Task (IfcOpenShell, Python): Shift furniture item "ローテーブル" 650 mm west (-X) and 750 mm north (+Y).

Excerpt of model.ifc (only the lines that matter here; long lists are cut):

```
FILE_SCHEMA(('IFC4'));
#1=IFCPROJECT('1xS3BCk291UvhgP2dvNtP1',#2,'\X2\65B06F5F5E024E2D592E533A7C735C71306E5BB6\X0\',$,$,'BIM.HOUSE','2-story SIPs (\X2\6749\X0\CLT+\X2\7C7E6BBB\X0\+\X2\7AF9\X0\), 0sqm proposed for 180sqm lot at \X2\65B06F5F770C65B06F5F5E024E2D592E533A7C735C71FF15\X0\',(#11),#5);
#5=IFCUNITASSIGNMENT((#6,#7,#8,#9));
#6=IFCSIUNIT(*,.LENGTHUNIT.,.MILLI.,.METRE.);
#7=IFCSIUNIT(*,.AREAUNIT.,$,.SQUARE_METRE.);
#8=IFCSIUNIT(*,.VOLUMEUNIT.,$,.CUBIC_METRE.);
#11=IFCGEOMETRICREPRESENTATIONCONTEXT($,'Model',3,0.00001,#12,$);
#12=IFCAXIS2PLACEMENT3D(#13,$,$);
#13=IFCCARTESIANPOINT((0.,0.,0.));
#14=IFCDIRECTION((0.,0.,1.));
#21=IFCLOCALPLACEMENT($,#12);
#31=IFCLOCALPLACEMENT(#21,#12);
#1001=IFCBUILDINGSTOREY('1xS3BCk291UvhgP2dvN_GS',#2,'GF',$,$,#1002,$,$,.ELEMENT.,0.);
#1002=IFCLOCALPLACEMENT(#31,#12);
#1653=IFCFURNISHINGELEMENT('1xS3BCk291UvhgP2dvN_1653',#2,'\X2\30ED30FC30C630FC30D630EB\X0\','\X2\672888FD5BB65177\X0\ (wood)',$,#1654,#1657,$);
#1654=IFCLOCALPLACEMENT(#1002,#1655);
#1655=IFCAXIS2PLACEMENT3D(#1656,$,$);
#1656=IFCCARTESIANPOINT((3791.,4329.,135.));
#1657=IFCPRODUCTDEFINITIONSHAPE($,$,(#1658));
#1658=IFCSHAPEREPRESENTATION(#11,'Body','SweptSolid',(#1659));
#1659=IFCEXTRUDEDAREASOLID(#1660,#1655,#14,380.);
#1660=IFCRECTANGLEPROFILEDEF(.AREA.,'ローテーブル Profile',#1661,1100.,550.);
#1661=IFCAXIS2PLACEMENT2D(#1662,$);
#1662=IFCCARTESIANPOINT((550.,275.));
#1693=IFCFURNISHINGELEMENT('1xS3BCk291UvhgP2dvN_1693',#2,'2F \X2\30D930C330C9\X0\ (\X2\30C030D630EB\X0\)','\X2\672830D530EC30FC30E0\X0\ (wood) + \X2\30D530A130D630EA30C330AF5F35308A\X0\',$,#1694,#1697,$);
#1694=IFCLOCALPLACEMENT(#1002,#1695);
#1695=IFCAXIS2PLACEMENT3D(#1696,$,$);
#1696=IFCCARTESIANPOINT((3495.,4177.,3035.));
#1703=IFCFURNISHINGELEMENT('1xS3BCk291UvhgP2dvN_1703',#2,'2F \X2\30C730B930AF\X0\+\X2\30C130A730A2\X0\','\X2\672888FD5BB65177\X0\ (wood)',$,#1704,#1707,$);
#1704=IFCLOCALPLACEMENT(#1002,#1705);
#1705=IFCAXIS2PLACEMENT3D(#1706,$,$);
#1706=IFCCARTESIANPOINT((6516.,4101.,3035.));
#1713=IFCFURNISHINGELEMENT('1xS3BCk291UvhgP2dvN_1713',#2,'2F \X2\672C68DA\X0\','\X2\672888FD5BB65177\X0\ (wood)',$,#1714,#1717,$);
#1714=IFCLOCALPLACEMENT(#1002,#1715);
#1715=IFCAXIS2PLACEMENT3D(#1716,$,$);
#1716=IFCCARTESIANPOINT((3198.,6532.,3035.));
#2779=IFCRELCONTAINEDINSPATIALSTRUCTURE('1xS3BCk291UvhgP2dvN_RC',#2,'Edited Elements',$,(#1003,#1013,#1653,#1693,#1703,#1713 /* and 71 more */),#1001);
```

```python
import ifcopenshell
import ifcopenshell.api.geometry
import ifcopenshell.util.placement
import ifcopenshell.util.unit

model = ifcopenshell.open("model.ifc")
unit_scale = ifcopenshell.util.unit.calculate_unit_scale(model)

item = model.by_id(1653)
matrix = ifcopenshell.util.placement.get_local_placement(item.ObjectPlacement)
matrix[0, 3] -= 0.65 / unit_scale
matrix[1, 3] += 0.75 / unit_scale
ifcopenshell.api.geometry.edit_object_placement(model, product=item, matrix=matrix, is_si=False)

print(ifcopenshell.util.placement.get_local_placement(item.ObjectPlacement).round(3) + 0.0)

model.write("model_rev.ifc")
```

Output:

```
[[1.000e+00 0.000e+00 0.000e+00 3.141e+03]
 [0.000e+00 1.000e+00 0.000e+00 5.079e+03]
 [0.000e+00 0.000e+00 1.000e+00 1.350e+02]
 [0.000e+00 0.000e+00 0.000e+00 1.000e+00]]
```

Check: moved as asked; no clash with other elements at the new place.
